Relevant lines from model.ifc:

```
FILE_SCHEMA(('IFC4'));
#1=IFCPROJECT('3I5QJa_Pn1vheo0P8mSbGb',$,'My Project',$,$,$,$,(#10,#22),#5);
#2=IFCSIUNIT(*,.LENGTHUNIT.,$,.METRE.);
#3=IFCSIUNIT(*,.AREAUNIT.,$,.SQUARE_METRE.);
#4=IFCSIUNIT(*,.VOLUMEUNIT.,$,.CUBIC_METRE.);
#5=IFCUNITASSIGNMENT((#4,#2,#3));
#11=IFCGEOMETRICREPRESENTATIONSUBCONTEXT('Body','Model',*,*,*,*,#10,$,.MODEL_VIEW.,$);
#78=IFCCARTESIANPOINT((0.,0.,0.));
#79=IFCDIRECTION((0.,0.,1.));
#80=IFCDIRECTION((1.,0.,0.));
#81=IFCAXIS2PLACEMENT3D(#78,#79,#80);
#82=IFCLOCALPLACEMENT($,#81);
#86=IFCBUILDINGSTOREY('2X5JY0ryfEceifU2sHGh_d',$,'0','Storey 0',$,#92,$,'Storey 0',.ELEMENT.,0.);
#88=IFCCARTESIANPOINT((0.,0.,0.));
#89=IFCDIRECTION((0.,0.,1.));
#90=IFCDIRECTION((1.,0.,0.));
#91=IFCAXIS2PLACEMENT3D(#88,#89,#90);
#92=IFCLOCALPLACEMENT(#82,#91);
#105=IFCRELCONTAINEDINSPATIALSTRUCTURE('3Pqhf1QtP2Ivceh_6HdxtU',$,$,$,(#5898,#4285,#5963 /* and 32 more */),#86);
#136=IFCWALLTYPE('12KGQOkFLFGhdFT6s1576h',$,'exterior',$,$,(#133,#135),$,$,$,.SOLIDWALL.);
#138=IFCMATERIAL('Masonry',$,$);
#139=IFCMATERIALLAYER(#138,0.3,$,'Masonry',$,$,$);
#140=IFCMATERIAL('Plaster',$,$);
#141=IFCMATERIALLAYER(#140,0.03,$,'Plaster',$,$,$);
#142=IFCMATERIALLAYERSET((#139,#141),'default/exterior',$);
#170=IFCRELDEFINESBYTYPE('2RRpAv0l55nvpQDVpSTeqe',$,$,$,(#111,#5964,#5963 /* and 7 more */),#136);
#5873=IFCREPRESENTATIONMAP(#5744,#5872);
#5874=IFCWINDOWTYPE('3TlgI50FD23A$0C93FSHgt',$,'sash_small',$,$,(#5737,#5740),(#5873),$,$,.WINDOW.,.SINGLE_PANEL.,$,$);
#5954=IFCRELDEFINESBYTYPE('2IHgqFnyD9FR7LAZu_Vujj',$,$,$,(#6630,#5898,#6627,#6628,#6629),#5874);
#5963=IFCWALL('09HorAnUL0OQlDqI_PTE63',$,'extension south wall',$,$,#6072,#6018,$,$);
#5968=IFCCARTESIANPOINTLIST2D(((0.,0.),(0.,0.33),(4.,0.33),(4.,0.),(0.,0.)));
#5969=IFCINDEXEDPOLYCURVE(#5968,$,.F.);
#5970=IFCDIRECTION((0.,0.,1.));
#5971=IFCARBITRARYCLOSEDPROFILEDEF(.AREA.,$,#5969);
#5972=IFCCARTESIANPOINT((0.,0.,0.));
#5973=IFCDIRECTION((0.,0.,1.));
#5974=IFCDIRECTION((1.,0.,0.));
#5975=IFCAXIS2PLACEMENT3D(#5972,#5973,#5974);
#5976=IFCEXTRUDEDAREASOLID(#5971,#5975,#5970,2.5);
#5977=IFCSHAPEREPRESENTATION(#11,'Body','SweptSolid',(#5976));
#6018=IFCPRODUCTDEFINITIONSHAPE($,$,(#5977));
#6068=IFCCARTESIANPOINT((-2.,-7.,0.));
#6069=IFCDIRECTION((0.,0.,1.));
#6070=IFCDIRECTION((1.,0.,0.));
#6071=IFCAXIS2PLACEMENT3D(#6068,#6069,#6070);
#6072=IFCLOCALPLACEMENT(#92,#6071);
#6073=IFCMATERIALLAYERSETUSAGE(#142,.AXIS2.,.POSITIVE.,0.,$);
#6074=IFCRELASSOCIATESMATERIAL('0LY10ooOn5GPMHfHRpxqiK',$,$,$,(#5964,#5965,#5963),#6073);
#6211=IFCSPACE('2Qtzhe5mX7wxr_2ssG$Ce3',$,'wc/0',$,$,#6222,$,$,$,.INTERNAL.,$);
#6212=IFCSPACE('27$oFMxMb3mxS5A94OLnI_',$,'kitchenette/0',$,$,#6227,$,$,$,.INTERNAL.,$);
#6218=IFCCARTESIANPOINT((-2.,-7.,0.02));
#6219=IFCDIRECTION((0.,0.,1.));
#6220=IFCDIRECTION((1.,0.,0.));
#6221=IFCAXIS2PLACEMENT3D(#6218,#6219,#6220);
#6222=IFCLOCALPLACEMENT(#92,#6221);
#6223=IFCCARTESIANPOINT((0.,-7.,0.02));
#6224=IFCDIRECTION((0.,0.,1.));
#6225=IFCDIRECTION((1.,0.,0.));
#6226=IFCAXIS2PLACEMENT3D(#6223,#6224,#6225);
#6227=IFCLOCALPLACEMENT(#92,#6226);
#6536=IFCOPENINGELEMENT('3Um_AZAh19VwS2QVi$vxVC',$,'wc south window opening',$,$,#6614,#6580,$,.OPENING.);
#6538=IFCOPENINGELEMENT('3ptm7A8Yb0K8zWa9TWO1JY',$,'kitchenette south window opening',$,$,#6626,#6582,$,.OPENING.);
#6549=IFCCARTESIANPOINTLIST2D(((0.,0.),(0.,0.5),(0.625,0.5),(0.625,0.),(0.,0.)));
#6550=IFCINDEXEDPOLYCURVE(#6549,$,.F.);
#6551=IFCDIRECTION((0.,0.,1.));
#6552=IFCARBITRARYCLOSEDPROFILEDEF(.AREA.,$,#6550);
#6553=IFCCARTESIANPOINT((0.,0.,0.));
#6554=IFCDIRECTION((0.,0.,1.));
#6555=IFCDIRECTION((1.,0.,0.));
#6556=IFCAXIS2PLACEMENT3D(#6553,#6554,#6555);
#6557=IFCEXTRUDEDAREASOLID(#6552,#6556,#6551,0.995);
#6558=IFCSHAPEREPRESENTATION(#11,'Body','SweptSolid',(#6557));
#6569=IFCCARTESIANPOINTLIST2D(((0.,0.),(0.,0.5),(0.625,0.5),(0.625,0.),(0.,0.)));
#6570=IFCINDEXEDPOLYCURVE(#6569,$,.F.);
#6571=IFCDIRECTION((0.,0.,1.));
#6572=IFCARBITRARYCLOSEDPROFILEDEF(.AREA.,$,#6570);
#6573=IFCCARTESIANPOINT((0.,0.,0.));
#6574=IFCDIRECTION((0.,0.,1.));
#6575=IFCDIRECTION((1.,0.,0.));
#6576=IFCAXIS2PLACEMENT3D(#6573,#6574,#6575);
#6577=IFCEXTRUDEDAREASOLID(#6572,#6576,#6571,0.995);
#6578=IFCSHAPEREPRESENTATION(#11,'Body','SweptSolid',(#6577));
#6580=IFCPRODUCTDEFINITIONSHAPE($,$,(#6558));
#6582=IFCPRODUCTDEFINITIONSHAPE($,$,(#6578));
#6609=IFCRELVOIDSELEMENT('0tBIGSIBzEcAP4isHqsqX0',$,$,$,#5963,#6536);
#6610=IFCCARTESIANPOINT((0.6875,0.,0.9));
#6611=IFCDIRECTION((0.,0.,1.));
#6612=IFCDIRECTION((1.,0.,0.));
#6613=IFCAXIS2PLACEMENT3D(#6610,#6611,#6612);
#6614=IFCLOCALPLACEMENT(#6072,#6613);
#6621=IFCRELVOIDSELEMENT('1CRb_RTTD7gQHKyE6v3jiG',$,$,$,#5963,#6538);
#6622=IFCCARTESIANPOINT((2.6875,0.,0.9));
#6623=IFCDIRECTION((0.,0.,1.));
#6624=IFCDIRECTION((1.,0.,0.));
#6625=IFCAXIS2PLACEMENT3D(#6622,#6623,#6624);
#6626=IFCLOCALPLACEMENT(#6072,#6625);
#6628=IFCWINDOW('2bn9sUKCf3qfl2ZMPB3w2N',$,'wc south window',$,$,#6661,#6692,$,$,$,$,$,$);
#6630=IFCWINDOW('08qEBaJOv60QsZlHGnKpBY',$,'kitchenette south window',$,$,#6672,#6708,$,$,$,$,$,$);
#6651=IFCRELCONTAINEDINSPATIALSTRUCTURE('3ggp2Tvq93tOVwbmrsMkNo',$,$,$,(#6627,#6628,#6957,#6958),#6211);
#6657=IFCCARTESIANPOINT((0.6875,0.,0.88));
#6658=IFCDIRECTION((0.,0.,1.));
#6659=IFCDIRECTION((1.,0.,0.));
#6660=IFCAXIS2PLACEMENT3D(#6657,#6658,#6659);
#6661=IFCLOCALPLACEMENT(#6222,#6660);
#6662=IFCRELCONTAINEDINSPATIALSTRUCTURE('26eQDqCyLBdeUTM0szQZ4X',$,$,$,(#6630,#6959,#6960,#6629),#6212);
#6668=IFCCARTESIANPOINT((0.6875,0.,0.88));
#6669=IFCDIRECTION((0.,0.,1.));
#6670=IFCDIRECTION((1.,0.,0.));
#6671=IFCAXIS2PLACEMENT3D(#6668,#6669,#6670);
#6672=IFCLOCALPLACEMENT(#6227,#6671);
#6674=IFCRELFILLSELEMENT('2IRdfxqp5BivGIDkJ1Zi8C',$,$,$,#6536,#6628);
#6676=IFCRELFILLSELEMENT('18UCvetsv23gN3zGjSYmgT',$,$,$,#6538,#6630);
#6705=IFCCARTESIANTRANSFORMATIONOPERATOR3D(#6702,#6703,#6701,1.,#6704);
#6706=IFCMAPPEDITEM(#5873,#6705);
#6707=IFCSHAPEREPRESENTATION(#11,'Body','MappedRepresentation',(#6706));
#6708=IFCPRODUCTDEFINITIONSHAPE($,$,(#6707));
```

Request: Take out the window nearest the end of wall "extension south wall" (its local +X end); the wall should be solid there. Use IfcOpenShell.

```python
import ifcopenshell
import ifcopenshell.api.feature
import ifcopenshell.api.root
import ifcopenshell.geom
import ifcopenshell.util.shape

model = ifcopenshell.open("model.ifc")
settings = ifcopenshell.geom.settings()


def volume(element):
    """Net volume in cubic metres, openings subtracted."""
    shape = ifcopenshell.geom.create_shape(settings, element)
    return ifcopenshell.util.shape.get_volume(shape.geometry)


window = model.by_guid("08qEBaJOv60QsZlHGnKpBY")
opening = window.FillsVoids[0].RelatingOpeningElement
wall = opening.VoidsElements[0].RelatingBuildingElement
before = volume(wall)

ifcopenshell.api.root.remove_product(model, product=window)
ifcopenshell.api.feature.remove_feature(model, feature=opening)

after = volume(wall)

print(f"wall volume {before:.3f} -> {after:.3f} m3")

model.write("model_v2.ifc")
```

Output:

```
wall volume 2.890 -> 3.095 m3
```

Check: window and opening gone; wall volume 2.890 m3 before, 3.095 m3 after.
